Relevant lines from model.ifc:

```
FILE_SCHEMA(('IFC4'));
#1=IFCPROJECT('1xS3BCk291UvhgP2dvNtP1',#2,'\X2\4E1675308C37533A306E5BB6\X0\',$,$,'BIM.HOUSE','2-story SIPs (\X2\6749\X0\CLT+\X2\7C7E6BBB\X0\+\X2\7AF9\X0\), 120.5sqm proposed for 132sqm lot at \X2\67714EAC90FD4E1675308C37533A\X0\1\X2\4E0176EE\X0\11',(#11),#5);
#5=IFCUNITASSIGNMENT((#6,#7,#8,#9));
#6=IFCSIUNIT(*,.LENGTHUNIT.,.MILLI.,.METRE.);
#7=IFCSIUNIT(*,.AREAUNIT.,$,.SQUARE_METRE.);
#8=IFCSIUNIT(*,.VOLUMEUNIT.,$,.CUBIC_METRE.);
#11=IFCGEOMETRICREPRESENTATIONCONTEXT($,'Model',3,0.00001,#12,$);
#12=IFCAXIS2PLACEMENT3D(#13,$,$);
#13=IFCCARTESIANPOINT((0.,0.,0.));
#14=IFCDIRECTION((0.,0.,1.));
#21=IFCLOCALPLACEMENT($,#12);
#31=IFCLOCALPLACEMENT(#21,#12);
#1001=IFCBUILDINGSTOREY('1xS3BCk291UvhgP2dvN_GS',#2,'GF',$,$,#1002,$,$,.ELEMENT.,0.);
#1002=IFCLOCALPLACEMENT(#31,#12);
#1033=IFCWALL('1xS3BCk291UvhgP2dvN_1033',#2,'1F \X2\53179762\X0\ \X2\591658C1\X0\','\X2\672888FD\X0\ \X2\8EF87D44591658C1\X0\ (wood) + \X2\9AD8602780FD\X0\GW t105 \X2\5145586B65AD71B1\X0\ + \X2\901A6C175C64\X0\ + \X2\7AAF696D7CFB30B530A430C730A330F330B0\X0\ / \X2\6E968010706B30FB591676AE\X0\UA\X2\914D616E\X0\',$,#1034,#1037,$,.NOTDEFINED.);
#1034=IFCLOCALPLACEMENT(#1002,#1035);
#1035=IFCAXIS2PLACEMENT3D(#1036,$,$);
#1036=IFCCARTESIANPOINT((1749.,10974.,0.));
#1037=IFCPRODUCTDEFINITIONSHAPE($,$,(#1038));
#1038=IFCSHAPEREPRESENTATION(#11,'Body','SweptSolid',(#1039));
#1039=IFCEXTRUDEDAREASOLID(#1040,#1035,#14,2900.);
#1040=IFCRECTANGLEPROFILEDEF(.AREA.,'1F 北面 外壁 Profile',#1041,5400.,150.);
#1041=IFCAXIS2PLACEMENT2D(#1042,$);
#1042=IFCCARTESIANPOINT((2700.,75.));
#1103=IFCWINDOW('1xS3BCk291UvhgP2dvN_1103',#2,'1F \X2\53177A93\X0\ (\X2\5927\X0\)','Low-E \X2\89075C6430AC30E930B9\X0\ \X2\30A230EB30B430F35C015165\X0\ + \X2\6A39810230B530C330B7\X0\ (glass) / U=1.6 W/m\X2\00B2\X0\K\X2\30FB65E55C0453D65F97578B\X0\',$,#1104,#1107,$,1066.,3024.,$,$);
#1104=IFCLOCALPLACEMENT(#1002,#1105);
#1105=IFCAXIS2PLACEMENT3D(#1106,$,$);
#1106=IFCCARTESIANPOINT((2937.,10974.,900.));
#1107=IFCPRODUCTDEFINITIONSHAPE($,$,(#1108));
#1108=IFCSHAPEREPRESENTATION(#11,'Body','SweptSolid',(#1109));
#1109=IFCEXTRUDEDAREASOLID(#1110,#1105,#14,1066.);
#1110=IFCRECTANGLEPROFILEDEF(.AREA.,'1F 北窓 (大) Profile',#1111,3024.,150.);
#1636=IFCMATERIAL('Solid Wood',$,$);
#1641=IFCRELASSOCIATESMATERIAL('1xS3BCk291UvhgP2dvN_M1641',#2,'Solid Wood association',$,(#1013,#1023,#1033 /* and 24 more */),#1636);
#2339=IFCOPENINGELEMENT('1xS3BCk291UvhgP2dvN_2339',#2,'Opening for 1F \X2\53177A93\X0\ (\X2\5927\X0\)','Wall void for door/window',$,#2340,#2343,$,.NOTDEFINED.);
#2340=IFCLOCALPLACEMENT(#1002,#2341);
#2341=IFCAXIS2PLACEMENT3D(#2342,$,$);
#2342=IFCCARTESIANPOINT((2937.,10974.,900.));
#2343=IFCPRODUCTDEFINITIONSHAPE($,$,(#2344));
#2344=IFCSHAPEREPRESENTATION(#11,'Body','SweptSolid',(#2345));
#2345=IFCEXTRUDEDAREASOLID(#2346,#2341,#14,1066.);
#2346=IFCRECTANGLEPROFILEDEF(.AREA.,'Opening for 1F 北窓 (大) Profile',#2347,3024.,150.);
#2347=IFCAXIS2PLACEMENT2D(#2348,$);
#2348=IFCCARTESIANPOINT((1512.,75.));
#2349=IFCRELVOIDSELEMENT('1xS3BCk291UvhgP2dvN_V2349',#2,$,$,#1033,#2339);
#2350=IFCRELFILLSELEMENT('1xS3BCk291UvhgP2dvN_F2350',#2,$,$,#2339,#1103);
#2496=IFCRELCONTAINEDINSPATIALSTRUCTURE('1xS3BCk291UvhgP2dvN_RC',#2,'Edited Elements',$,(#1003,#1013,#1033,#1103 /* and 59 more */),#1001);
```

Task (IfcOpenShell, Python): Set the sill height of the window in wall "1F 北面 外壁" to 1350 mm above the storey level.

```python
import numpy as np
import ifcopenshell
import ifcopenshell.api.geometry
import ifcopenshell.geom
import ifcopenshell.util.element
import ifcopenshell.util.placement
import ifcopenshell.util.shape
import ifcopenshell.util.unit

model = ifcopenshell.open("model.ifc")
unit_scale = ifcopenshell.util.unit.calculate_unit_scale(model)

window = model.by_guid("1xS3BCk291UvhgP2dvN_1103")
opening = window.FillsVoids[0].RelatingOpeningElement
storey = ifcopenshell.util.element.get_container(window, ifc_class="IfcBuildingStorey")
level = ifcopenshell.util.placement.get_local_placement(storey.ObjectPlacement)[2, 3]

# The opening's origin need not be at the sill, so measure its lowest point.
shape = ifcopenshell.geom.create_shape(ifcopenshell.geom.settings(), opening)
bottom = ifcopenshell.util.shape.get_shape_bottom_elevation(shape, shape.geometry) / unit_scale
dz = level + 1.35 / unit_scale - bottom

shift = np.array([0.0, 0.0, dz])
# The window is not placed relative to its opening, so move both.
for product in (opening, window):
    matrix = ifcopenshell.util.placement.get_local_placement(product.ObjectPlacement)
    matrix[:3, 3] += shift
    ifcopenshell.api.geometry.edit_object_placement(model, product=product, matrix=matrix, is_si=False)

print(f"moved by {dz * unit_scale:+.3f} m")

model.write("model_rev.ifc")
```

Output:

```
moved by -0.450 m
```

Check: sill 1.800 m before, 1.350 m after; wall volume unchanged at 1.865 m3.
